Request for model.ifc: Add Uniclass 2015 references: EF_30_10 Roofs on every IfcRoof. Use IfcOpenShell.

First a look at what the model holds.

```python
import ifcopenshell

model = ifcopenshell.open("model.ifc")
print(model.schema)
print("classifications:", [c.Name for c in model.by_type("IfcClassification")])
for ifc_class in ("IfcDoor", "IfcRoof", "IfcStair", "IfcWall", "IfcWindow"):
    print(ifc_class, len(model.by_type(ifc_class)))
```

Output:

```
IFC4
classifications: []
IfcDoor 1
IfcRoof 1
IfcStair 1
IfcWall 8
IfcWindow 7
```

```python
import ifcopenshell
import ifcopenshell.api.classification

model = ifcopenshell.open("model.ifc")

system = ifcopenshell.api.classification.add_classification(model, classification="Uniclass 2015")

codes = {
    "IfcRoof": ("EF_30_10", "Roofs"),
}
for ifc_class, (code, name) in codes.items():
    products = model.by_type(ifc_class)
    ifcopenshell.api.classification.add_reference(
        model, products=products, classification=system, identification=code, name=name
    )
    print(code, len(products))

model.write("model-out.ifc")
```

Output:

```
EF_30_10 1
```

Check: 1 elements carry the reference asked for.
